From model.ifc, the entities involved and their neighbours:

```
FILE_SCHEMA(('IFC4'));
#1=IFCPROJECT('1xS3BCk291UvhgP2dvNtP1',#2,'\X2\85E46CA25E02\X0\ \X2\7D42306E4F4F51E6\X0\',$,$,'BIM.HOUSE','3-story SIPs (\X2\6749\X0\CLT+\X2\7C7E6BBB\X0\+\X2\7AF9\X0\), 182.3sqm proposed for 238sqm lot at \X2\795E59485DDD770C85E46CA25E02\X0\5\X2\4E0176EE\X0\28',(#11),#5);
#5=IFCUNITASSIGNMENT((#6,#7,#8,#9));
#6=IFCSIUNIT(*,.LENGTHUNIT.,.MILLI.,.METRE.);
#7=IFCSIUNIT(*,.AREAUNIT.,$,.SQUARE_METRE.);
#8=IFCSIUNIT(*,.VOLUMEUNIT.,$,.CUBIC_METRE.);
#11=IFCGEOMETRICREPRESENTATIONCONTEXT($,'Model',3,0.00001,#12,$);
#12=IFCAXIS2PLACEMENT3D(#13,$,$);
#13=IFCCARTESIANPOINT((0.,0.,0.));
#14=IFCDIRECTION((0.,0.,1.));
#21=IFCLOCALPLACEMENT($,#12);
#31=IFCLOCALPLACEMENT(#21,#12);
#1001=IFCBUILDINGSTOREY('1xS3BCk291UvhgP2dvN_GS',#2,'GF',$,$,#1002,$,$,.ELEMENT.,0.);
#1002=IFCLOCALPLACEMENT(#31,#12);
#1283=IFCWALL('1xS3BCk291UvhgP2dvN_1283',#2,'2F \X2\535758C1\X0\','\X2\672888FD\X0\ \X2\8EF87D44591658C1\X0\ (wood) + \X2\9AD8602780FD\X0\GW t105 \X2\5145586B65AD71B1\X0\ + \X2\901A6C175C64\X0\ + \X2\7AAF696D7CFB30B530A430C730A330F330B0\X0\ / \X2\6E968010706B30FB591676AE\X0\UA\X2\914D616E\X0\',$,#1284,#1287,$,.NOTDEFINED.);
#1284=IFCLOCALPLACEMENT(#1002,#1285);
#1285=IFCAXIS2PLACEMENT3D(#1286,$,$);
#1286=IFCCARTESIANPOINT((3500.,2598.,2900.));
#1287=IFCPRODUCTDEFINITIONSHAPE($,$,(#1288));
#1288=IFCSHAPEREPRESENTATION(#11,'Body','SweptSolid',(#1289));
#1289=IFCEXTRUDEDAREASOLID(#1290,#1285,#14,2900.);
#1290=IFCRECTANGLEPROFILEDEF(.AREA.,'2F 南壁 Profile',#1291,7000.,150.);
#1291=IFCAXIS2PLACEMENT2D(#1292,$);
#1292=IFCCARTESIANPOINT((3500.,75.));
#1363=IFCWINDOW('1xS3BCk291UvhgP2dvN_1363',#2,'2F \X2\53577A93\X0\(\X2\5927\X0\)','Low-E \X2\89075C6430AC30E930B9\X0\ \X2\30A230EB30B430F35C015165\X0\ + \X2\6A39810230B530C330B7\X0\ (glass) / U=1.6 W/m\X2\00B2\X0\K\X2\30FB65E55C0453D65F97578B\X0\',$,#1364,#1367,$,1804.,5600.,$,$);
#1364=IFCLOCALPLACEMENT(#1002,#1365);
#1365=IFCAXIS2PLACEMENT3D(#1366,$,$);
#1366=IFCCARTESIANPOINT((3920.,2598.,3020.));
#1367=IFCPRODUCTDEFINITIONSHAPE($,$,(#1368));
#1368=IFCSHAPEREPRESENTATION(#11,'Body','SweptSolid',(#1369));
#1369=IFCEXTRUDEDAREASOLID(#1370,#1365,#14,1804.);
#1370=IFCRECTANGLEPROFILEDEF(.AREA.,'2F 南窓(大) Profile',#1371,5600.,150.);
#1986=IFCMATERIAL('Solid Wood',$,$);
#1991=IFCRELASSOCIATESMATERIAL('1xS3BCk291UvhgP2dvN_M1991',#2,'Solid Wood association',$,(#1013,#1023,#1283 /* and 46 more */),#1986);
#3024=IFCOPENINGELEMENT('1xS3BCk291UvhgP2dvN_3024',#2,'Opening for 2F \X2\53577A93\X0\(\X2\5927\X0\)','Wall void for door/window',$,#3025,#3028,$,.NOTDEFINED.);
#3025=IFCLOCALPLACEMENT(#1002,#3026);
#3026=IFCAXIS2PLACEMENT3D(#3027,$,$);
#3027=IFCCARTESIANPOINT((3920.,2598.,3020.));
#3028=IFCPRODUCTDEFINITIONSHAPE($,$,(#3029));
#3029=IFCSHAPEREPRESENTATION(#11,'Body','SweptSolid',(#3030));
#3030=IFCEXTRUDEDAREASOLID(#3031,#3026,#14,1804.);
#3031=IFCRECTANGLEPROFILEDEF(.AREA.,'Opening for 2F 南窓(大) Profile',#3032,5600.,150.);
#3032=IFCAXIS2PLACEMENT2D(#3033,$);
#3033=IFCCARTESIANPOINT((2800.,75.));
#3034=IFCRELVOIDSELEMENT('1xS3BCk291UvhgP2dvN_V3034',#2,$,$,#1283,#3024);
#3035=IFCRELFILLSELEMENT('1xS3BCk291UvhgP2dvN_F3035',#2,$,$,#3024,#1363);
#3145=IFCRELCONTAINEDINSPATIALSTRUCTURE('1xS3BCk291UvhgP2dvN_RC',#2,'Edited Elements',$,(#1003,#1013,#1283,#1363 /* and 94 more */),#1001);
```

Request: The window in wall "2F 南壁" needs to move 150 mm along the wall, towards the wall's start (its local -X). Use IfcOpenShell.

```python
import ifcopenshell
import ifcopenshell.api.geometry
import ifcopenshell.util.placement
import ifcopenshell.util.unit

model = ifcopenshell.open("model.ifc")
unit_scale = ifcopenshell.util.unit.calculate_unit_scale(model)

window = model.by_guid("1xS3BCk291UvhgP2dvN_1363")
opening = window.FillsVoids[0].RelatingOpeningElement
wall = opening.VoidsElements[0].RelatingBuildingElement

wall_matrix = ifcopenshell.util.placement.get_local_placement(wall.ObjectPlacement)
shift = wall_matrix[:3, 0] * -0.15 / unit_scale
before = ifcopenshell.util.placement.get_local_placement(window.ObjectPlacement)[:3, 3].copy()

# The window is not placed relative to its opening, so move both.
for product in (opening, window):
    matrix = ifcopenshell.util.placement.get_local_placement(product.ObjectPlacement)
    matrix[:3, 3] += shift
    ifcopenshell.api.geometry.edit_object_placement(model, product=product, matrix=matrix, is_si=False)

after = ifcopenshell.util.placement.get_local_placement(window.ObjectPlacement)[:3, 3]
print("window moved by", (after - before).round(3) + 0.0)

model.write("model_edited.ifc")
```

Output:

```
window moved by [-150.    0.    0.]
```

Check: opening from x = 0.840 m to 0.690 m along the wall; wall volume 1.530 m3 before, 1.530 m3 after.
